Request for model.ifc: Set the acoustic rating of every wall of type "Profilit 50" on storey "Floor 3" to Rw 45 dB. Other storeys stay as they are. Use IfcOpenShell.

First a look at what the model holds.

```python
import ifcopenshell
import ifcopenshell.util.element

model = ifcopenshell.open("model.ifc")
print(model.schema)
storey = next(s for s in model.by_type("IfcBuildingStorey") if s.Name == "Floor 3")
walls = [e for e in ifcopenshell.util.element.get_decomposition(storey) if e.is_a("IfcWall")]
seen = {}
for e in walls:
    element_type = ifcopenshell.util.element.get_type(e)
    key = (element_type.Name if element_type != e and element_type else None, ifcopenshell.util.element.get_pset(e, "Pset_WallCommon", "AcousticRating"))
    seen[key] = seen.get(key, 0) + 1
for (name, value), count in sorted(seen.items(), key=str):
    print(count, "x", name, "|", value)
```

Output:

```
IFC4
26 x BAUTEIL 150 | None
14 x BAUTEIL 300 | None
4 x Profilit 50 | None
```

```python
import ifcopenshell
import ifcopenshell.api.pset
import ifcopenshell.util.element

model = ifcopenshell.open("model.ifc")

storey = next(s for s in model.by_type("IfcBuildingStorey") if s.Name == "Floor 3")
walls = [e for e in ifcopenshell.util.element.get_decomposition(storey) if e.is_a("IfcWall")]

count = 0
for e in walls:
    element_type = ifcopenshell.util.element.get_type(e)
    if element_type in (None, e) or element_type.Name != "Profilit 50":
        continue
    # add_pset returns the element's existing set when there is one.
    pset = ifcopenshell.api.pset.add_pset(model, product=e, name="Pset_WallCommon")
    ifcopenshell.api.pset.edit_pset(model, pset=pset, properties={"AcousticRating": "Rw 45 dB"})
    count += 1

print(count, "walls updated")

model.write("model_updated.ifc")
```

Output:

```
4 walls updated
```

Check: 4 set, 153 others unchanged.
